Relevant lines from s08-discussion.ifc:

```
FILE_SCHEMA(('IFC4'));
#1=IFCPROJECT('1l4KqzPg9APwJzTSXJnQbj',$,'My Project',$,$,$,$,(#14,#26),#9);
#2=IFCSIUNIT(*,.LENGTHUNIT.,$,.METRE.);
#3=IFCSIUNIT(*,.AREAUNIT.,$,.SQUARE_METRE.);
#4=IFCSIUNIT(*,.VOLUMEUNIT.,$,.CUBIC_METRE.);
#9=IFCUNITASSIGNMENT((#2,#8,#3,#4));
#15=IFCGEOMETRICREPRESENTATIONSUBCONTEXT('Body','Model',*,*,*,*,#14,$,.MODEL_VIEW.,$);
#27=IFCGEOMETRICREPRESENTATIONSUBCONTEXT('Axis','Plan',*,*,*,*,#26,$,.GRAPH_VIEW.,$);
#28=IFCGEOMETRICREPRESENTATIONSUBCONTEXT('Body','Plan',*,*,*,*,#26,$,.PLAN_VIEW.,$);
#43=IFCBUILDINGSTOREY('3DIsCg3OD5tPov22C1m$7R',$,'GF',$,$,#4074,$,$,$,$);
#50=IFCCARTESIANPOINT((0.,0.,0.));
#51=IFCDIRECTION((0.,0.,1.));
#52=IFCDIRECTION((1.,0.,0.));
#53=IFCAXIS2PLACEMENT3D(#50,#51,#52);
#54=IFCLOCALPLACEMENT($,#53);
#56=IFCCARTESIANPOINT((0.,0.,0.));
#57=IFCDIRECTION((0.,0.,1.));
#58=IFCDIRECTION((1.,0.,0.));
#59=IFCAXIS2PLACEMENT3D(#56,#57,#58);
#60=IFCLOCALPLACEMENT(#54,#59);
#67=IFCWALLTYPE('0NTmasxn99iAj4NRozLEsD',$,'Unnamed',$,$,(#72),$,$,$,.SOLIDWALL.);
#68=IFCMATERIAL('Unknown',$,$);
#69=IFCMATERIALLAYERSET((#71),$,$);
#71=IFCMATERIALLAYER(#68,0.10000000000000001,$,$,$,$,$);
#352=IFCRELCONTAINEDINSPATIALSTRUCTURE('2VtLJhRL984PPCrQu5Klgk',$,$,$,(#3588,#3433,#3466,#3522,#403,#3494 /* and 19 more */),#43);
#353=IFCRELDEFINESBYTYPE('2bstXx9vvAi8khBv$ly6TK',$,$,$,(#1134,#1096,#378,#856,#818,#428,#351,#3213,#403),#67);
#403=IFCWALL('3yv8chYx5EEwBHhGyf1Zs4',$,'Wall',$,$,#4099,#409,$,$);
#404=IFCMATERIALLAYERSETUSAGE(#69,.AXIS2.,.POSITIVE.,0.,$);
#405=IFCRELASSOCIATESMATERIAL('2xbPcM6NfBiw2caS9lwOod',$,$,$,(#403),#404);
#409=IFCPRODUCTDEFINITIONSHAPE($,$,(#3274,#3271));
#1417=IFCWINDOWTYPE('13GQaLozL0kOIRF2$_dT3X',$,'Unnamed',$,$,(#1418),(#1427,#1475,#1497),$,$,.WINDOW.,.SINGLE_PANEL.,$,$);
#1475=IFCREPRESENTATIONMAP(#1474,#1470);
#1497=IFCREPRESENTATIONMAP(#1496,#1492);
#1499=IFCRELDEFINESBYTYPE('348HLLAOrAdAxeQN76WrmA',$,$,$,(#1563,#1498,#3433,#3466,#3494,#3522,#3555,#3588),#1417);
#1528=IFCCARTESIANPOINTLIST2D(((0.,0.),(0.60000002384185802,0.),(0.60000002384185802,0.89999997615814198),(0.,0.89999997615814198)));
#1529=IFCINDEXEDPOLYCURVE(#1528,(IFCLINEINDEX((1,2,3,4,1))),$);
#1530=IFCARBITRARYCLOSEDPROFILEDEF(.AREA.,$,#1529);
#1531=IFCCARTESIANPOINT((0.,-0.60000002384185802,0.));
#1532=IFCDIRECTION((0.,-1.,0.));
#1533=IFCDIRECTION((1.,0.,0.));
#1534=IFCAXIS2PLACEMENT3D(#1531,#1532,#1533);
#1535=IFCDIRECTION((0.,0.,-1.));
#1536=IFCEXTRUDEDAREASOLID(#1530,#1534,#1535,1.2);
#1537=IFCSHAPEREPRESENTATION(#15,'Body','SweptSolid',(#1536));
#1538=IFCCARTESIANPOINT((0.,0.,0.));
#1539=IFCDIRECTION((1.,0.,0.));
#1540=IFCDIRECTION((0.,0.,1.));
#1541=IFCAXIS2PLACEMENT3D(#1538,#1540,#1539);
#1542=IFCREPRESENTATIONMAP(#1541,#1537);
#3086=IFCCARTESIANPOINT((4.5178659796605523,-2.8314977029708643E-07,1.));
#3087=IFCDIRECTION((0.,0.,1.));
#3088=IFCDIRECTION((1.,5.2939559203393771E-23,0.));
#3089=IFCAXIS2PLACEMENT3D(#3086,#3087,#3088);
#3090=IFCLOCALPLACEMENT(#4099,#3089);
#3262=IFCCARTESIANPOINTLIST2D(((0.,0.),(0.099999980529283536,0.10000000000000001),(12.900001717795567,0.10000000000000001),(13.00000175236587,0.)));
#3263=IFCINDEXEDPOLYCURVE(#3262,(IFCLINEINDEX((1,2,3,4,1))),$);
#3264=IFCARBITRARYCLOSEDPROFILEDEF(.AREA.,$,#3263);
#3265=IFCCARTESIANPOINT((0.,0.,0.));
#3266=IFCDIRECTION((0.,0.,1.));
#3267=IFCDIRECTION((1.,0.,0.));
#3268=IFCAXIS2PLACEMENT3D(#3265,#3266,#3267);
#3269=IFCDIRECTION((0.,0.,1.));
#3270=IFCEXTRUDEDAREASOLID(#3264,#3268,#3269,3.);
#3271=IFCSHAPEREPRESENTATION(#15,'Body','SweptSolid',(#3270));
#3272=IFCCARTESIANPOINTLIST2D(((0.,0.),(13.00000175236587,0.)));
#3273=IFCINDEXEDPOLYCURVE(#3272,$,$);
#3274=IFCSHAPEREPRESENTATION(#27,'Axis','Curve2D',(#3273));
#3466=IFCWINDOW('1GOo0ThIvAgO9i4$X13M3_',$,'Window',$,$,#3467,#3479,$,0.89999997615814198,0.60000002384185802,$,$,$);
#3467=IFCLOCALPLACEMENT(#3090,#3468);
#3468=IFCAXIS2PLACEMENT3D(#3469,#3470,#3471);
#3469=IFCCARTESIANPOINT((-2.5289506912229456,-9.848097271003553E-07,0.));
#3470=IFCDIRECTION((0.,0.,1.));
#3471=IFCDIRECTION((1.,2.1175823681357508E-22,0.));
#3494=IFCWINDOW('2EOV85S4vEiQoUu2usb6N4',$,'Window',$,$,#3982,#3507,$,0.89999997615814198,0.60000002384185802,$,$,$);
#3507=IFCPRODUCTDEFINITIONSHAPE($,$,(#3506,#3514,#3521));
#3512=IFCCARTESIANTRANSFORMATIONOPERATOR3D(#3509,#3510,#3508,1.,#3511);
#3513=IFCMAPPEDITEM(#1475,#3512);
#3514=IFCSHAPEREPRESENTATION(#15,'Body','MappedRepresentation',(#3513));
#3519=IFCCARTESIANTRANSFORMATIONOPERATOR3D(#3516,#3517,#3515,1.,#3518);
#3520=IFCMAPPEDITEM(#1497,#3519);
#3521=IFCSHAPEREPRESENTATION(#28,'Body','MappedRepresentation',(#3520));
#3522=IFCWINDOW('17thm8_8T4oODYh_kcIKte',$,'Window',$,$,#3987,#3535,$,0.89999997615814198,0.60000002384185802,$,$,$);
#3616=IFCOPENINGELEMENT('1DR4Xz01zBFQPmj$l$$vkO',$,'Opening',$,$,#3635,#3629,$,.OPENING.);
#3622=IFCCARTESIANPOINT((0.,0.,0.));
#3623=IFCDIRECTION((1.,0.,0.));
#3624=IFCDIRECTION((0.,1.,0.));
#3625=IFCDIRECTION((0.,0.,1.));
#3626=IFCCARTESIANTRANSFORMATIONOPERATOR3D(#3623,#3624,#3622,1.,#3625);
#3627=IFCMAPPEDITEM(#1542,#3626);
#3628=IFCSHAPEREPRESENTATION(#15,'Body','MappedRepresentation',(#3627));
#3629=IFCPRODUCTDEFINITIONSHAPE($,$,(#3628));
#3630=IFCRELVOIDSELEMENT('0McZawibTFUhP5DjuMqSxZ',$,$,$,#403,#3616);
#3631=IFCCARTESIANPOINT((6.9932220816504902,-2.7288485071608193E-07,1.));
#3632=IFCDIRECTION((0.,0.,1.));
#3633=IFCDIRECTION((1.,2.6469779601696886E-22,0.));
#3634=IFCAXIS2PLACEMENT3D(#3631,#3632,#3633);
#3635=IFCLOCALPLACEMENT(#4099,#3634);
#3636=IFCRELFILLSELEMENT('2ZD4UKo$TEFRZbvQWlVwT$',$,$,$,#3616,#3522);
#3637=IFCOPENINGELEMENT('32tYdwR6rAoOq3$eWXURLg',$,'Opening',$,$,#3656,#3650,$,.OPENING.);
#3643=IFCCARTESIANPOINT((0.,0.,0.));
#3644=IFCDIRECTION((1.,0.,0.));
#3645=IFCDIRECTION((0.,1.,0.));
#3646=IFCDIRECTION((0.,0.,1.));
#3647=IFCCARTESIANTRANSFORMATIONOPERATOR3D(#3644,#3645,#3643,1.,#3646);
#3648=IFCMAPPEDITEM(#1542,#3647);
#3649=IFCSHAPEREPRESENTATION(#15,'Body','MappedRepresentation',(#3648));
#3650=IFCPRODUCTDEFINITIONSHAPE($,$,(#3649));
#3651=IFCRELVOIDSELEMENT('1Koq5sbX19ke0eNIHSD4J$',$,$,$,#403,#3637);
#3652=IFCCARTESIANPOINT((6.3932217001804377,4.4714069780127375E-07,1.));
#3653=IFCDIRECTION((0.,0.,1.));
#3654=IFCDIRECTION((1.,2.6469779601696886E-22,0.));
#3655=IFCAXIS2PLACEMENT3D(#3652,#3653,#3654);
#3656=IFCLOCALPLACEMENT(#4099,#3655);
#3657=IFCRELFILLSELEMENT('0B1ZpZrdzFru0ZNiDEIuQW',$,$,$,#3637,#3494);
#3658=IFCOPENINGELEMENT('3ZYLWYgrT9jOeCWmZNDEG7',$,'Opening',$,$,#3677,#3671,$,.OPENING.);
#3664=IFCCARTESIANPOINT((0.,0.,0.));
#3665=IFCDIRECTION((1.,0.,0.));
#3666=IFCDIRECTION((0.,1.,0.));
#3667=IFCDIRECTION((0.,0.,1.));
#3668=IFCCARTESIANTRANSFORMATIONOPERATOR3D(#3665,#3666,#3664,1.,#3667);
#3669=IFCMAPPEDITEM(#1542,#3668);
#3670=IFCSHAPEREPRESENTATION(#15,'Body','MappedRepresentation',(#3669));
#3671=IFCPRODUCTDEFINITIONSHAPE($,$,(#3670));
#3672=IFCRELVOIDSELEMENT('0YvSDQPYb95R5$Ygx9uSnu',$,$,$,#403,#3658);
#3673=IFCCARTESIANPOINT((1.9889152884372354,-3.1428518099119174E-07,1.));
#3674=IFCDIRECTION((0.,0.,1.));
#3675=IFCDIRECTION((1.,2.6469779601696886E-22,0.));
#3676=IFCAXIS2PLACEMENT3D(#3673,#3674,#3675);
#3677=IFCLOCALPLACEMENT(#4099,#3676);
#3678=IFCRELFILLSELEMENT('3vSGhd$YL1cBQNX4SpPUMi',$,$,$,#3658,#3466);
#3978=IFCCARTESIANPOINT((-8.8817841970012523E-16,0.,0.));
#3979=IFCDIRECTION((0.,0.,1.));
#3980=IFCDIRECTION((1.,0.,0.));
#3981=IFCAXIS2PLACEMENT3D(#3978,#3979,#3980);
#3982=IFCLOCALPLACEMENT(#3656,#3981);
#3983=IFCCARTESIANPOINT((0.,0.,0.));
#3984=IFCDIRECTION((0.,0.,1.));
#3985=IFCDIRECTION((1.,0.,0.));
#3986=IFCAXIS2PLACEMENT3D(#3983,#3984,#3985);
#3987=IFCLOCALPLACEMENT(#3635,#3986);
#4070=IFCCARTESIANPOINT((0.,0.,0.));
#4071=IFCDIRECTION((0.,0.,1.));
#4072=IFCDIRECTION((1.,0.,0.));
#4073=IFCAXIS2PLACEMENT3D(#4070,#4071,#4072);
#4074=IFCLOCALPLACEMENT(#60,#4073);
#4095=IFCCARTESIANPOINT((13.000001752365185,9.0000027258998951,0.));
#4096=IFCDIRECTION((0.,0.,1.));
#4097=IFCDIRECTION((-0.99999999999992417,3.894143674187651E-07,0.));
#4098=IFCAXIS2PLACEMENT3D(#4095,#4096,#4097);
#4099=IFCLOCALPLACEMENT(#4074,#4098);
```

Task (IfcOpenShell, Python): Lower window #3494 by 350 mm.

```python
import numpy as np
import ifcopenshell
import ifcopenshell.api.geometry
import ifcopenshell.util.placement
import ifcopenshell.util.unit

model = ifcopenshell.open("s08-discussion.ifc")
unit_scale = ifcopenshell.util.unit.calculate_unit_scale(model)

window = model.by_id(3494)
opening = window.FillsVoids[0].RelatingOpeningElement
dz = -0.35 / unit_scale

shift = np.array([0.0, 0.0, dz])
# The window is placed relative to its opening, so it follows when the opening moves.
matrix = ifcopenshell.util.placement.get_local_placement(opening.ObjectPlacement)
matrix[:3, 3] += shift
ifcopenshell.api.geometry.edit_object_placement(
    model, product=opening, matrix=matrix, is_si=False, should_transform_children=True
)

print(f"moved by {dz * unit_scale:+.3f} m")

model.write("s08-discussion_rev.ifc")
```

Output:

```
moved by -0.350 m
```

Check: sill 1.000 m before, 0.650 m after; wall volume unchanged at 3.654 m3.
